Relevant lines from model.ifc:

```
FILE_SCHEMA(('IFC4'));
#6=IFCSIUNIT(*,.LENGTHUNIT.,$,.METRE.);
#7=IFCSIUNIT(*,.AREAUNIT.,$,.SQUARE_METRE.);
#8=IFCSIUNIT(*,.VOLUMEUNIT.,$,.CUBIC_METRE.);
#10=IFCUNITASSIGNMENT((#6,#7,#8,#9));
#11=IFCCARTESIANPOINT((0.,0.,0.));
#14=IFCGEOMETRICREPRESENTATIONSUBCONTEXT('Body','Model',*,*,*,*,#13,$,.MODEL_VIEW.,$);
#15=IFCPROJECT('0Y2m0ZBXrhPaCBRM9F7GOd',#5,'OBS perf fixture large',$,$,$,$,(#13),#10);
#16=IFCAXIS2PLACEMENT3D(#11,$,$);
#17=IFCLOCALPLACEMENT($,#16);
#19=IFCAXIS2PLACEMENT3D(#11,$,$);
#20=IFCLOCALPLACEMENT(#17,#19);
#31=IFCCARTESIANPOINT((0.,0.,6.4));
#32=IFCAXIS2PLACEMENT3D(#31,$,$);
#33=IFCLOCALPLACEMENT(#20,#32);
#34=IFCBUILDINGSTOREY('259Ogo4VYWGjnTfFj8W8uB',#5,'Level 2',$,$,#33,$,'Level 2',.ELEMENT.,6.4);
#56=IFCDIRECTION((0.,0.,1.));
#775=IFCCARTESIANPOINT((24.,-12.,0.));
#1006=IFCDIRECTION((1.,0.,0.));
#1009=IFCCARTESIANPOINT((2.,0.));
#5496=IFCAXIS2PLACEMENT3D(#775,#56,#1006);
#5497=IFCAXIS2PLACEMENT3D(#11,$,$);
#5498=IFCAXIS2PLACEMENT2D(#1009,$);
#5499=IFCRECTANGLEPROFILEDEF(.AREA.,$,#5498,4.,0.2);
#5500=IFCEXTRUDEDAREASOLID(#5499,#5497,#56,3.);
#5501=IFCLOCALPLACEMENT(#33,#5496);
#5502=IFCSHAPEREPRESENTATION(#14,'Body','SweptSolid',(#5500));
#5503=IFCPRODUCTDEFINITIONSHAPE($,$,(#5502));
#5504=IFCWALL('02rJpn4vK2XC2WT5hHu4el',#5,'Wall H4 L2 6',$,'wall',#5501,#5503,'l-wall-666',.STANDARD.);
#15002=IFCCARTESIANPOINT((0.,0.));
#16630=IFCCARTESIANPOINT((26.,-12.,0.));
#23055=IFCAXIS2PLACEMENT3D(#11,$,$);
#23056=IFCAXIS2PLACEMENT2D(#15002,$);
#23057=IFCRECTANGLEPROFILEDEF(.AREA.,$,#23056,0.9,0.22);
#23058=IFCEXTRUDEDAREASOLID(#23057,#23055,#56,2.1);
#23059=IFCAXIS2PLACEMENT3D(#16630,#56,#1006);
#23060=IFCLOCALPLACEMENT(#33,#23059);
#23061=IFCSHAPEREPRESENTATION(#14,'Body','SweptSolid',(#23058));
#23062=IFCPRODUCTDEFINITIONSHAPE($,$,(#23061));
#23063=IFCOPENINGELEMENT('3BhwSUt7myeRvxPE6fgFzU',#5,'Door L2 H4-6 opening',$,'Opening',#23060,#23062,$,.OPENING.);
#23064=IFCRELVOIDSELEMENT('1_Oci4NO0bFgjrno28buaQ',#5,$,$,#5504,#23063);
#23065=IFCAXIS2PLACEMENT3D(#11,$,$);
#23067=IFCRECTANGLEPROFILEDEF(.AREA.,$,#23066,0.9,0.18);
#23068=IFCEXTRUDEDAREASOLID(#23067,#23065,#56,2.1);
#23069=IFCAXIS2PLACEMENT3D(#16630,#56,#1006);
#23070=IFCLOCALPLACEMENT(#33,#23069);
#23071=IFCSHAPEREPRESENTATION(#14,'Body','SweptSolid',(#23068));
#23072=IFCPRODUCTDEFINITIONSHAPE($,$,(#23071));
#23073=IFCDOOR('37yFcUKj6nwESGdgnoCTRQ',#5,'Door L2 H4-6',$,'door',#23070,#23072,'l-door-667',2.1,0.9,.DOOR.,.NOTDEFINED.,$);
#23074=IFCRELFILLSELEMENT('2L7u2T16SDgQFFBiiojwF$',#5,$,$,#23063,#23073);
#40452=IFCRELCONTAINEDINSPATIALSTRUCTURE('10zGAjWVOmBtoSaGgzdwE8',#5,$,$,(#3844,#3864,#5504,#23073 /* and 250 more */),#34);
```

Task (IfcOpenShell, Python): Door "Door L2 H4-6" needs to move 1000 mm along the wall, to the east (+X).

```python
import ifcopenshell
import ifcopenshell.api.geometry
import ifcopenshell.util.placement
import ifcopenshell.util.unit

model = ifcopenshell.open("model.ifc")
unit_scale = ifcopenshell.util.unit.calculate_unit_scale(model)

door = model.by_id(23073)
opening = door.FillsVoids[0].RelatingOpeningElement
wall = opening.VoidsElements[0].RelatingBuildingElement

wall_matrix = ifcopenshell.util.placement.get_local_placement(wall.ObjectPlacement)
shift = wall_matrix[:3, 0] * 1 / unit_scale
before = ifcopenshell.util.placement.get_local_placement(door.ObjectPlacement)[:3, 3].copy()

# The door is not placed relative to its opening, so move both.
for product in (opening, door):
    matrix = ifcopenshell.util.placement.get_local_placement(product.ObjectPlacement)
    matrix[:3, 3] += shift
    ifcopenshell.api.geometry.edit_object_placement(model, product=product, matrix=matrix, is_si=False)

after = ifcopenshell.util.placement.get_local_placement(door.ObjectPlacement)[:3, 3]
print("door moved by", (after - before).round(3) + 0.0)

model.write("model_rev.ifc")
```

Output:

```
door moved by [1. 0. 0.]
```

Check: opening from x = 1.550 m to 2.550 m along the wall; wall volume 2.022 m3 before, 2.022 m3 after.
